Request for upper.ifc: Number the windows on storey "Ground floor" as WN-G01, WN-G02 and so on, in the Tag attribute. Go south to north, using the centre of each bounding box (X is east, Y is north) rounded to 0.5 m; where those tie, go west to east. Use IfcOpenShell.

First a look at what the model holds.

```python
import ifcopenshell
import ifcopenshell.util.element
import ifcopenshell.util.placement

model = ifcopenshell.open("upper.ifc")
print(model.schema)
storey = next(s for s in model.by_type("IfcBuildingStorey") if s.Name == "Ground floor")
windows = [e for e in ifcopenshell.util.element.get_decomposition(storey) if e.is_a("IfcWindow")]
for e in sorted(windows, key=lambda e: e.id()):
    origin = ifcopenshell.util.placement.get_local_placement(e.ObjectPlacement)[:3, 3]
    print(e.id(), e.Tag, e.Name, origin.round(2) + 0.0, sep=" | ")
```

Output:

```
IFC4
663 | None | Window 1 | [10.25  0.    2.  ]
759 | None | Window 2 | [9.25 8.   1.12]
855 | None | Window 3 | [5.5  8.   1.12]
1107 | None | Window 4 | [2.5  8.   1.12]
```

```python
import ifcopenshell
import ifcopenshell.geom
import ifcopenshell.util.element
import ifcopenshell.util.shape

model = ifcopenshell.open("upper.ifc")
settings = ifcopenshell.geom.settings()
settings.set("use-world-coords", True)


def centre(element):
    shape = ifcopenshell.geom.create_shape(settings, element)
    return ifcopenshell.util.shape.get_bbox_centroid(shape.geometry)


storey = next(s for s in model.by_type("IfcBuildingStorey") if s.Name == "Ground floor")
windows = [e for e in ifcopenshell.util.element.get_decomposition(storey) if e.is_a("IfcWindow")]

# Insertion points can sit at a corner or the storey origin, so sort by the geometry (in metres).
centres = {e: centre(e) for e in windows}
windows.sort(key=lambda e: (round(centres[e][1] / 0.5), centres[e][0]))

for i, e in enumerate(windows, start=1):
    number = f"WN-G{i:02d}"
    e.Tag = number
    print(e.id(), number)

model.write("upper_rev.ifc")
```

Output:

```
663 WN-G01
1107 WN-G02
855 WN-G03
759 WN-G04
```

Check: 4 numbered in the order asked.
